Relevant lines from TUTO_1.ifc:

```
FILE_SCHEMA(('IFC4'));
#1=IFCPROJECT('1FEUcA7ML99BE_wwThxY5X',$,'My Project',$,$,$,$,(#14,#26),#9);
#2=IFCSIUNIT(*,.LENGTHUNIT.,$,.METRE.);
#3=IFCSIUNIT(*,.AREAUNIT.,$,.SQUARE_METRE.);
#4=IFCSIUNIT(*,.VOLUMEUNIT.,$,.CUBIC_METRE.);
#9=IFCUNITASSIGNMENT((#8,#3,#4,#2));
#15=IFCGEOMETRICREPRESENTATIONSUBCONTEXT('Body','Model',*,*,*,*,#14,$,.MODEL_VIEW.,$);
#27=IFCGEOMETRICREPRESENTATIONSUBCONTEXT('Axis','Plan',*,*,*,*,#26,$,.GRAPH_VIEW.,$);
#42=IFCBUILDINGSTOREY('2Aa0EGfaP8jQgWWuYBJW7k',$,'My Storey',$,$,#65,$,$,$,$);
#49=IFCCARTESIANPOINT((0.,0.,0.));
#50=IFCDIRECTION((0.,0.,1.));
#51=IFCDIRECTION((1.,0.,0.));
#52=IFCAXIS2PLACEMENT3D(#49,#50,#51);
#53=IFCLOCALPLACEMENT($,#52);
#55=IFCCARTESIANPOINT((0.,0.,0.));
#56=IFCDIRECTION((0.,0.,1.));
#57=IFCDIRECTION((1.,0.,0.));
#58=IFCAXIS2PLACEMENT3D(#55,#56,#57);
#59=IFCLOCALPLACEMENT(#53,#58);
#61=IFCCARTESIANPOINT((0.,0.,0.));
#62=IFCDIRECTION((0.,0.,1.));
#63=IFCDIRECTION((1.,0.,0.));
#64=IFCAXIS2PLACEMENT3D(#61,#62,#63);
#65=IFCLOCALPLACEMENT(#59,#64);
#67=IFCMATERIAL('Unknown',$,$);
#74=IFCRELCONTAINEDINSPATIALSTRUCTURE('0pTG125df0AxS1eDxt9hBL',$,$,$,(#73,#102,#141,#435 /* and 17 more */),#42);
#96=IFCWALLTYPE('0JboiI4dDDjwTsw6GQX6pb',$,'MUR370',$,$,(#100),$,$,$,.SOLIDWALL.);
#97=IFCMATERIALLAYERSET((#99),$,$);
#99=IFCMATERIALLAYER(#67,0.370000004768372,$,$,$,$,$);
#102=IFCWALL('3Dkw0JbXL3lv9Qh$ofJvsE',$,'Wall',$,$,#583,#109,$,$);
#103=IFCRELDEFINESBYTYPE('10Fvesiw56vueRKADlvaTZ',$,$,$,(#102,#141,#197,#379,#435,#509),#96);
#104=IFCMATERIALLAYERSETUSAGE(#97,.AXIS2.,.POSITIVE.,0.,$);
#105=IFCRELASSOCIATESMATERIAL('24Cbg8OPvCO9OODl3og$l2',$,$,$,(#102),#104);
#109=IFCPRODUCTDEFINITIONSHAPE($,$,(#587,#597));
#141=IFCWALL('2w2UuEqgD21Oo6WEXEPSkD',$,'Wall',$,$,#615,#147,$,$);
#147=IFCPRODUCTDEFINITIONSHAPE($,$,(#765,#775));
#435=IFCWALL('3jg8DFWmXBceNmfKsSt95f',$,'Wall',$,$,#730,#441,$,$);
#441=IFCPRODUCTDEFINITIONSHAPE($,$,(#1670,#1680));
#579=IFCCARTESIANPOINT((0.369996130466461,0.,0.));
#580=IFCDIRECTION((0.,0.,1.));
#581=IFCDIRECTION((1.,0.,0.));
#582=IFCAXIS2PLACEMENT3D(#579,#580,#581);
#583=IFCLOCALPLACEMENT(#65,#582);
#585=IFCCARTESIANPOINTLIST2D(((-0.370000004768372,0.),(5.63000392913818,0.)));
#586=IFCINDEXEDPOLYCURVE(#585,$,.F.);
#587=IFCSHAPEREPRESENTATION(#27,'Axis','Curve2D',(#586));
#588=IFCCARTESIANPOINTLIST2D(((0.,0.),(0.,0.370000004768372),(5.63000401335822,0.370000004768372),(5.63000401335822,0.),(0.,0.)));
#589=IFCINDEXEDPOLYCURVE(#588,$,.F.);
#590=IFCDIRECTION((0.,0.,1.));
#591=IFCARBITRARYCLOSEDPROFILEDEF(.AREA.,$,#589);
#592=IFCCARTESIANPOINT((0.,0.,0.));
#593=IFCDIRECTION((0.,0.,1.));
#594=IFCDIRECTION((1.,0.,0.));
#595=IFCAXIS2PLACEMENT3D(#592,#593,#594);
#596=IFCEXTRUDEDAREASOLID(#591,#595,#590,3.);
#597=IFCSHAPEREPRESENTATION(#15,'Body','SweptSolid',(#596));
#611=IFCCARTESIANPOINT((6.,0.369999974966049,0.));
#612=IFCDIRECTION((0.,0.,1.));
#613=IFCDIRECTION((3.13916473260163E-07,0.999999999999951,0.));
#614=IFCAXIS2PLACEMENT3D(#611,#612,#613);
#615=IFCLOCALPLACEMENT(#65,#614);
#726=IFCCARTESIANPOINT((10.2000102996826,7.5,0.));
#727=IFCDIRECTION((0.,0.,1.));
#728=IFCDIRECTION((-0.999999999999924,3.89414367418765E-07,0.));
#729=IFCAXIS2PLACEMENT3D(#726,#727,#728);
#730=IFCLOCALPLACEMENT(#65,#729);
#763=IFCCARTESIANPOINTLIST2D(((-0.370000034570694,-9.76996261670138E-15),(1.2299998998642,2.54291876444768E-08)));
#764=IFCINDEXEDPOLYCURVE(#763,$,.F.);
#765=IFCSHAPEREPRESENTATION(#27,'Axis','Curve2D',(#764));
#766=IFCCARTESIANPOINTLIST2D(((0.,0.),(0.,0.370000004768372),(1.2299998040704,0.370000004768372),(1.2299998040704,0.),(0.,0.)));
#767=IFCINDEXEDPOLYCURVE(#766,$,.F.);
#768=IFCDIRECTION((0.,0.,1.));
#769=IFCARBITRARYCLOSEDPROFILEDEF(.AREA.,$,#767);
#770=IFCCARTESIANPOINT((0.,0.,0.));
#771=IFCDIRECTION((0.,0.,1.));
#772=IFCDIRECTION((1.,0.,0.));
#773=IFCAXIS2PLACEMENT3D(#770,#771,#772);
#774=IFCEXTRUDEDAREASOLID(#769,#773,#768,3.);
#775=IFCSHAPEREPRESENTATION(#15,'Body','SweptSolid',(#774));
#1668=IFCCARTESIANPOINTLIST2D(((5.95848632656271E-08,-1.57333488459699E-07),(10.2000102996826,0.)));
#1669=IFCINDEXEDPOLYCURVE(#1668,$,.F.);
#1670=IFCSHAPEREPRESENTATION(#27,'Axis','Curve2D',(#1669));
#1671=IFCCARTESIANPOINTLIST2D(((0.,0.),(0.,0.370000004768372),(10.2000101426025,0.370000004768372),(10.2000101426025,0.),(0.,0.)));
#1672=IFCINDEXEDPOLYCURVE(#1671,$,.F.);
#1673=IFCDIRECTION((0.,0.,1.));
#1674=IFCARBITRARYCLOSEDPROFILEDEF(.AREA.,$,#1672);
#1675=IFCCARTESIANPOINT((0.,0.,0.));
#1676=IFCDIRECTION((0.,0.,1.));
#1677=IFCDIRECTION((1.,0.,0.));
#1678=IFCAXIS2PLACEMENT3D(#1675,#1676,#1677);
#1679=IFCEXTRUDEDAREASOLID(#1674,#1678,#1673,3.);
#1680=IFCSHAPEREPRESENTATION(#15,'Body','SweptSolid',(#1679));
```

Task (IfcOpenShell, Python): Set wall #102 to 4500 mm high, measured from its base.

```python
import ifcopenshell
import ifcopenshell.geom
import ifcopenshell.util.representation
import ifcopenshell.util.shape

model = ifcopenshell.open("TUTO_1.ifc")
settings = ifcopenshell.geom.settings()


def volume(element):
    """Net volume in cubic metres, openings subtracted."""
    shape = ifcopenshell.geom.create_shape(settings, element)
    return ifcopenshell.util.shape.get_volume(shape.geometry)


wall = model.by_id(102)
before = volume(wall)

body = ifcopenshell.util.representation.get_representation(wall, "Model", "Body")
solid = body.Items[0]
old_height = solid.Depth
solid.Depth = 4.5
after = volume(wall)

print(f"height {old_height:g} -> {solid.Depth:g}, volume {before:.3f} -> {after:.3f} m3")

model.write("TUTO_1_updated.ifc")
```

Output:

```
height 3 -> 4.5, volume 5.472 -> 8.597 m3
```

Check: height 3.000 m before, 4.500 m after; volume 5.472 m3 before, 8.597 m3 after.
